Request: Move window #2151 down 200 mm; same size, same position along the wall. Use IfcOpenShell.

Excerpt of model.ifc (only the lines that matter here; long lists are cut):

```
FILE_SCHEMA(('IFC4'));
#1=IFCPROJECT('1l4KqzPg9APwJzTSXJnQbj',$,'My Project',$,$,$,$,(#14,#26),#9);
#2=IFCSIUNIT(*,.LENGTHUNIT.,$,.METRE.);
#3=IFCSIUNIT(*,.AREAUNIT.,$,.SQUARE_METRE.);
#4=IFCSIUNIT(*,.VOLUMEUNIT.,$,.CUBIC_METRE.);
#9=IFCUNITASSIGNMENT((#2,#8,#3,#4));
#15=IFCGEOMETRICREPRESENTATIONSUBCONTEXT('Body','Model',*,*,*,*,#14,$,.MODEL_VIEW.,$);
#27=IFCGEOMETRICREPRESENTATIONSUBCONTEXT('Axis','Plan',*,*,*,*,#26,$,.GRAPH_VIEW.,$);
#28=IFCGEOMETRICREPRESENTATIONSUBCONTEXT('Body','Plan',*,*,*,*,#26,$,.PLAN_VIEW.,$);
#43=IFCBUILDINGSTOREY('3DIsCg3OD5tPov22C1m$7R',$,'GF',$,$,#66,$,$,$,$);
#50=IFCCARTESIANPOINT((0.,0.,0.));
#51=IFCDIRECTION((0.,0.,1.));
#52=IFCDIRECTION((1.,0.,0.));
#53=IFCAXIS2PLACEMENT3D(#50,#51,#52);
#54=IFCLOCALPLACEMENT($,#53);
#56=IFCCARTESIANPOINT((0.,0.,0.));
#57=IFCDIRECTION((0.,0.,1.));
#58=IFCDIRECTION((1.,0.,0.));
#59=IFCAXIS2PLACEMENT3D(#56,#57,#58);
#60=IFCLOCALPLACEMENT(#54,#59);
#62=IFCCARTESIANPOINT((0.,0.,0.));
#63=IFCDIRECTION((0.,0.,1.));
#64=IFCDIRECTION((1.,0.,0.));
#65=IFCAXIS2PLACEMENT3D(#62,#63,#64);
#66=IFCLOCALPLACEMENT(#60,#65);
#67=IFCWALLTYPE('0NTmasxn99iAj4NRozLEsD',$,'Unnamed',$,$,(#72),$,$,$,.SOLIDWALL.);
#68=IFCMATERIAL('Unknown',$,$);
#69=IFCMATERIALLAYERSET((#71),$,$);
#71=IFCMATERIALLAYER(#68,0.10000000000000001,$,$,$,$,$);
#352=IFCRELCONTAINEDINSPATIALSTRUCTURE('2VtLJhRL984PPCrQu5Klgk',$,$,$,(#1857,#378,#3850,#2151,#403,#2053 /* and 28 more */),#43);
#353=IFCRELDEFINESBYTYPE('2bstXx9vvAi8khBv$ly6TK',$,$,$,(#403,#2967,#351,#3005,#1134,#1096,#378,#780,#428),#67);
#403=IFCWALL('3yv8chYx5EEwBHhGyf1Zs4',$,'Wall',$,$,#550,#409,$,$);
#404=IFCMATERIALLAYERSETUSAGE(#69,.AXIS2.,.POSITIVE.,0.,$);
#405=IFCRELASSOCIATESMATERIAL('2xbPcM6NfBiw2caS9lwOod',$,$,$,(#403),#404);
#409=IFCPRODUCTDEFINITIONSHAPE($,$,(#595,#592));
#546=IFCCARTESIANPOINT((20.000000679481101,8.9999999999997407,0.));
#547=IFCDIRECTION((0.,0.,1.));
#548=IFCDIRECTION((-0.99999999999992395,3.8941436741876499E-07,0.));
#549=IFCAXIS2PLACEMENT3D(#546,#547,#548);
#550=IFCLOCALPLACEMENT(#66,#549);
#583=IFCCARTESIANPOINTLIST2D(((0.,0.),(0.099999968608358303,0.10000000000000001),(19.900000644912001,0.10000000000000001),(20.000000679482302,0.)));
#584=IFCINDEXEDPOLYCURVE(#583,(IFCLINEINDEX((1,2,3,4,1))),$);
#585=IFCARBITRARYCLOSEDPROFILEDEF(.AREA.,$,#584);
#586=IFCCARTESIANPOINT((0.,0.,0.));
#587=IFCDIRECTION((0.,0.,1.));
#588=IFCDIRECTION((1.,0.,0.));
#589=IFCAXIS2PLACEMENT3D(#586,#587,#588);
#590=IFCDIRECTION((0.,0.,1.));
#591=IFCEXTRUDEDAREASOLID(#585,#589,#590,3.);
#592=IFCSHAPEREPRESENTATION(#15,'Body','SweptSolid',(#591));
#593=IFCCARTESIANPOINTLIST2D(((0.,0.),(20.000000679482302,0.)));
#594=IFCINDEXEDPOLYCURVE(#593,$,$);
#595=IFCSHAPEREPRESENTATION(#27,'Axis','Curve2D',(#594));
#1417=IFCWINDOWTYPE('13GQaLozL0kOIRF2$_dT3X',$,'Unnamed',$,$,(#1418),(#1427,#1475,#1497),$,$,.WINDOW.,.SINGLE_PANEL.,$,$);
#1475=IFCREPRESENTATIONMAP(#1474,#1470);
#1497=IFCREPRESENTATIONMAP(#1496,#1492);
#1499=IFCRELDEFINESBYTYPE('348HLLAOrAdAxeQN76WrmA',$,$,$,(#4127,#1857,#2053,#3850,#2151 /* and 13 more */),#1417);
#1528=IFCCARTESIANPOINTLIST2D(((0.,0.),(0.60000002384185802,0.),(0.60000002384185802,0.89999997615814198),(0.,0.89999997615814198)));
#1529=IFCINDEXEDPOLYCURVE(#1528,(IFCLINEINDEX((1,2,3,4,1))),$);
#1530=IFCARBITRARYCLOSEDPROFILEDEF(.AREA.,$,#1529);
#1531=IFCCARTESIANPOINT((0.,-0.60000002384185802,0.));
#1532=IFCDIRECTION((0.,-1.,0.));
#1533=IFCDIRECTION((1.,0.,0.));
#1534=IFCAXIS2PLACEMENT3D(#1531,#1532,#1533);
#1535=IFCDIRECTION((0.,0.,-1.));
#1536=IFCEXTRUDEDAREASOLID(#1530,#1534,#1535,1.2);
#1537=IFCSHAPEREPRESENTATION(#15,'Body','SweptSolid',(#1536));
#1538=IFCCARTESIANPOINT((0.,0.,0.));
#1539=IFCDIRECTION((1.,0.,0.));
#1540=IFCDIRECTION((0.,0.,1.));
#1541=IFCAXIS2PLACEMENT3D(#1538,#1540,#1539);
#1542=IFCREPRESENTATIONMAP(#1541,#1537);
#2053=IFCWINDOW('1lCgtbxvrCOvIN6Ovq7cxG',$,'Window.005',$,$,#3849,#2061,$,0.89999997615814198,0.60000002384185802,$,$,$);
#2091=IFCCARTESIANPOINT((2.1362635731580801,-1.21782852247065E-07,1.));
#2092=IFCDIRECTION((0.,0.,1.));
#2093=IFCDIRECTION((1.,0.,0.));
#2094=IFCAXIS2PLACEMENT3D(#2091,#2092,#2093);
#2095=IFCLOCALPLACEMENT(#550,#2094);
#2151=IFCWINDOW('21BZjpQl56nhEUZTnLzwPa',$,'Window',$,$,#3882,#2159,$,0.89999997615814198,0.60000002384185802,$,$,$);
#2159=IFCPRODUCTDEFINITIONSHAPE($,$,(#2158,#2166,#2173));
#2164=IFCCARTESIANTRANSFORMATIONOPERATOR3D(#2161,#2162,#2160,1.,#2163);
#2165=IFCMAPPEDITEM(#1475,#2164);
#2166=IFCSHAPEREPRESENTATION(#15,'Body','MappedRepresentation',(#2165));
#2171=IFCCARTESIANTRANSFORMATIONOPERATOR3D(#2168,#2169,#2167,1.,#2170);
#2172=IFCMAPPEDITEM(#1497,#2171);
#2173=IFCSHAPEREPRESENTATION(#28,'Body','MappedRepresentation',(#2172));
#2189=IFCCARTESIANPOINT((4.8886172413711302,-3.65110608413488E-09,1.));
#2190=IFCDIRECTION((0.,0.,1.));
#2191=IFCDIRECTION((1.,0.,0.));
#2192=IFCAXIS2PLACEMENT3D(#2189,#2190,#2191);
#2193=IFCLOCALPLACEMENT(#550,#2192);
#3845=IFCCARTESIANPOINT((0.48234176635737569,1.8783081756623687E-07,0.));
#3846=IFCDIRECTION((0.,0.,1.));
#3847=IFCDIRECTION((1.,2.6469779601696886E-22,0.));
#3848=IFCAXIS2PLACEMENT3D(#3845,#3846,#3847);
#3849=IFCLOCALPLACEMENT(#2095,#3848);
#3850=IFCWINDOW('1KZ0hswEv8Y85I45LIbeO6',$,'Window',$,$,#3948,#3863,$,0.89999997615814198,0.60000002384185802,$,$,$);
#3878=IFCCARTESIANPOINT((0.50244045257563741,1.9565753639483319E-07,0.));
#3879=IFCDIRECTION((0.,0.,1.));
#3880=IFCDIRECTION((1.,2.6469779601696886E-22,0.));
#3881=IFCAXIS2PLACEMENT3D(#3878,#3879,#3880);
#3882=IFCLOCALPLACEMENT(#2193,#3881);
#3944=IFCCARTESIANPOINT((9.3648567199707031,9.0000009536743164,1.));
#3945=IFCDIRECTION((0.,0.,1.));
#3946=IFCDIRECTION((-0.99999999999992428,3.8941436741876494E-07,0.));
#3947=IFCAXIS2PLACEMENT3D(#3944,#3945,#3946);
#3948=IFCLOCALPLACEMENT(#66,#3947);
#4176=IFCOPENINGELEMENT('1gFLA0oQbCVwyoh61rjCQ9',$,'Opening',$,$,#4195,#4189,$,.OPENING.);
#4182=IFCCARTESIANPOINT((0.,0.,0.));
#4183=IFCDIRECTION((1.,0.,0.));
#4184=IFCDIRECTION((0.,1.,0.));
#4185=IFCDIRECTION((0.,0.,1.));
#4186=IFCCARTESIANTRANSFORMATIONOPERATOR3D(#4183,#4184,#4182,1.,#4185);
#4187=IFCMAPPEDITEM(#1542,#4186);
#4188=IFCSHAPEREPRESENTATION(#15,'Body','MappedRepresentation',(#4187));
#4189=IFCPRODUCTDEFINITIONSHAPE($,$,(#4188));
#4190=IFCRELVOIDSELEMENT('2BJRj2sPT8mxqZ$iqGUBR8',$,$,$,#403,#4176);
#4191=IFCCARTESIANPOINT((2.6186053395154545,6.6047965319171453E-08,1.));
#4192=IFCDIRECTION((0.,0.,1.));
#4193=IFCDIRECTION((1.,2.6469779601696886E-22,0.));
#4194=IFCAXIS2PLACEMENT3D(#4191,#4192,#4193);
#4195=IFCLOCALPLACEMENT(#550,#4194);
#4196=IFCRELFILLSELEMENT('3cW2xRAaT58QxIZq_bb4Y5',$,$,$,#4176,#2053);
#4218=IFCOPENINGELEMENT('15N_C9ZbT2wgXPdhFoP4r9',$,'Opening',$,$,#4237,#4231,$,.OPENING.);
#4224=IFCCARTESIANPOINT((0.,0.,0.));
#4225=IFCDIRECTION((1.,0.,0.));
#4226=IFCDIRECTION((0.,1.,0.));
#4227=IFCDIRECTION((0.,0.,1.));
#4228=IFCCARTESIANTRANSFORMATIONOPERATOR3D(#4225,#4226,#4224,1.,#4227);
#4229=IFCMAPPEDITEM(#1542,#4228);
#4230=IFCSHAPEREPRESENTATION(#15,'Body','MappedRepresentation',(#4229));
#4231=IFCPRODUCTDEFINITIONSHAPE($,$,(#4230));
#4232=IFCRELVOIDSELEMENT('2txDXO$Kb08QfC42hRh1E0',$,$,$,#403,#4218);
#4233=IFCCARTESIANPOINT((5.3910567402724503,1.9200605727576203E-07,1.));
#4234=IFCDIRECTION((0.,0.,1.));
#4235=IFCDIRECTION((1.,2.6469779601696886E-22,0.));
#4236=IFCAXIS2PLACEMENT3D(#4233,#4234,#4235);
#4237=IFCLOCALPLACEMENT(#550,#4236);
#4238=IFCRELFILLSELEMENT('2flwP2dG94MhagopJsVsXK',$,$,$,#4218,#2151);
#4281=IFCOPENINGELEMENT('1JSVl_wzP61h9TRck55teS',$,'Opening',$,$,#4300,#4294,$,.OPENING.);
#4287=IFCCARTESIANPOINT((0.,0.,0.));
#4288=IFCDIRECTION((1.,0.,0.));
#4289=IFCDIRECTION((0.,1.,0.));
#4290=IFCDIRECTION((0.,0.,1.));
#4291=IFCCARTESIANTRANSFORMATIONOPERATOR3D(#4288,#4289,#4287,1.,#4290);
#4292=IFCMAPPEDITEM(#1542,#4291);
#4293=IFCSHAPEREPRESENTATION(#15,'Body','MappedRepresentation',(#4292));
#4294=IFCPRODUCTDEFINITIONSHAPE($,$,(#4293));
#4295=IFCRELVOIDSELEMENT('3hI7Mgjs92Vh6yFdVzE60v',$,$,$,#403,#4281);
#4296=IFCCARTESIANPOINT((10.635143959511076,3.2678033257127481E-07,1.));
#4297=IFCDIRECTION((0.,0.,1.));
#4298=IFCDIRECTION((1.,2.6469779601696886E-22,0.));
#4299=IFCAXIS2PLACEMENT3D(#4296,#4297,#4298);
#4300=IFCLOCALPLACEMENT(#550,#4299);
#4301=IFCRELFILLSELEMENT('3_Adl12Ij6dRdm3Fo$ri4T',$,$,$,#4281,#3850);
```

```python
import numpy as np
import ifcopenshell
import ifcopenshell.api.geometry
import ifcopenshell.util.placement
import ifcopenshell.util.unit

model = ifcopenshell.open("model.ifc")
unit_scale = ifcopenshell.util.unit.calculate_unit_scale(model)

window = model.by_id(2151)
opening = window.FillsVoids[0].RelatingOpeningElement
dz = -0.2 / unit_scale

shift = np.array([0.0, 0.0, dz])
# The window is not placed relative to its opening, so move both.
for product in (opening, window):
    matrix = ifcopenshell.util.placement.get_local_placement(product.ObjectPlacement)
    matrix[:3, 3] += shift
    ifcopenshell.api.geometry.edit_object_placement(model, product=product, matrix=matrix, is_si=False)

print(f"moved by {dz * unit_scale:+.3f} m")

model.write("model_v2.ifc")
```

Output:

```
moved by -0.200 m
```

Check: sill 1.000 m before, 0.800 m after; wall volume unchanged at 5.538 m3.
